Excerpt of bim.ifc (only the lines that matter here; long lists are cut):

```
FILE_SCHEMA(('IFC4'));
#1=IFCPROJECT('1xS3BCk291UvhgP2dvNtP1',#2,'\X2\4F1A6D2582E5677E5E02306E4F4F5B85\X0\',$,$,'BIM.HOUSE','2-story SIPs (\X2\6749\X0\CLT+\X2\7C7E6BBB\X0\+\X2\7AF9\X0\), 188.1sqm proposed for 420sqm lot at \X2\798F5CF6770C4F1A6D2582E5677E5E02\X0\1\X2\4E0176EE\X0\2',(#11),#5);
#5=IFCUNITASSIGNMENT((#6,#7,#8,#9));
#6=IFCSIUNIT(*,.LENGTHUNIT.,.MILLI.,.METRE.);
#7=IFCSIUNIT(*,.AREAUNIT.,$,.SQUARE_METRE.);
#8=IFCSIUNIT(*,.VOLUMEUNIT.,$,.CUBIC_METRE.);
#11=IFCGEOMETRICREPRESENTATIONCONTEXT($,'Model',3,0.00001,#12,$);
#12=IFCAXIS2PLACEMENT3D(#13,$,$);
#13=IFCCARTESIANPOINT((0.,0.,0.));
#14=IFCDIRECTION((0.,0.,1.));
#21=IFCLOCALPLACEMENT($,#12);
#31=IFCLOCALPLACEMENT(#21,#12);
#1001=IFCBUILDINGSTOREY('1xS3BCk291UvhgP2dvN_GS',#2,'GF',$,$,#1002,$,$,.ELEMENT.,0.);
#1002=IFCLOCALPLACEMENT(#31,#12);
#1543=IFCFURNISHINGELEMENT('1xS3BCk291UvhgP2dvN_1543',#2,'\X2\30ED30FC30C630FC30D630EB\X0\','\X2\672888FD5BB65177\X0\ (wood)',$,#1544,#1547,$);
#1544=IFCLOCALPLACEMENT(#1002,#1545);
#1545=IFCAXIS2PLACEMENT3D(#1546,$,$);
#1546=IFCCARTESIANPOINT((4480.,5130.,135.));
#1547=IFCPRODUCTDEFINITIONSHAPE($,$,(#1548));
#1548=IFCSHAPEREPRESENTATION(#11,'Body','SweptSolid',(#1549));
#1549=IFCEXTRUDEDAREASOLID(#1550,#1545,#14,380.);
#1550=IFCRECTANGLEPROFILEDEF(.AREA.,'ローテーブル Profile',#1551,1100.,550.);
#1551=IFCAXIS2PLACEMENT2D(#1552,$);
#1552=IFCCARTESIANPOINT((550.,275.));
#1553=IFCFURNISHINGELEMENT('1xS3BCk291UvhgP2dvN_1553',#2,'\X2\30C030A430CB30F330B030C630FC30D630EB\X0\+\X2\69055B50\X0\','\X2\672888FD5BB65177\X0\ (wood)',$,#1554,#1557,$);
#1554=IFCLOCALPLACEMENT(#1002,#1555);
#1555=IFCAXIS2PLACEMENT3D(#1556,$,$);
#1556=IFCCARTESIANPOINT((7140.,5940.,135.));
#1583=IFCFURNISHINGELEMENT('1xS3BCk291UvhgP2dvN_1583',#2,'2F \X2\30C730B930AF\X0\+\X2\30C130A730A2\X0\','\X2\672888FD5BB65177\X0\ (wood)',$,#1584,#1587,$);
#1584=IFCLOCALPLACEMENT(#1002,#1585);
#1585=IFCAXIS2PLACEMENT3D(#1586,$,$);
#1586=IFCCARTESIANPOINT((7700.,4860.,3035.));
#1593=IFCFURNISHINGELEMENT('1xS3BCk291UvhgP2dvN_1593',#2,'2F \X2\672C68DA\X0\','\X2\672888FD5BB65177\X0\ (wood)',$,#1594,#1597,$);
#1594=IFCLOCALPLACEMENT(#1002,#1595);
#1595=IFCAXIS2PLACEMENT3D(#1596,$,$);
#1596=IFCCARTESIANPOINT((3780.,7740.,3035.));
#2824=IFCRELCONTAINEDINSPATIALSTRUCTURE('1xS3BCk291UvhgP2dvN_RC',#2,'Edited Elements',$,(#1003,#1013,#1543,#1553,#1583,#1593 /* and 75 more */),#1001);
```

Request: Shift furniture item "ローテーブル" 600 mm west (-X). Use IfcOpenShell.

```python
import ifcopenshell
import ifcopenshell.api.geometry
import ifcopenshell.util.placement

model = ifcopenshell.open("bim.ifc")

item = model.by_id(1543)
matrix = ifcopenshell.util.placement.get_local_placement(item.ObjectPlacement)
matrix[0, 3] -= 600.0
ifcopenshell.api.geometry.edit_object_placement(model, product=item, matrix=matrix, is_si=False)

print(ifcopenshell.util.placement.get_local_placement(item.ObjectPlacement).round(3) + 0.0)

model.write("bim_updated.ifc")
```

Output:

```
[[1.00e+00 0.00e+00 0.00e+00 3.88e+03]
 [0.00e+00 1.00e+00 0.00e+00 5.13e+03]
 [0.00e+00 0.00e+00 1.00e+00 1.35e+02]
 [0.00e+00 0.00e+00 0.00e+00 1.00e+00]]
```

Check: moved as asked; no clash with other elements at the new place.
